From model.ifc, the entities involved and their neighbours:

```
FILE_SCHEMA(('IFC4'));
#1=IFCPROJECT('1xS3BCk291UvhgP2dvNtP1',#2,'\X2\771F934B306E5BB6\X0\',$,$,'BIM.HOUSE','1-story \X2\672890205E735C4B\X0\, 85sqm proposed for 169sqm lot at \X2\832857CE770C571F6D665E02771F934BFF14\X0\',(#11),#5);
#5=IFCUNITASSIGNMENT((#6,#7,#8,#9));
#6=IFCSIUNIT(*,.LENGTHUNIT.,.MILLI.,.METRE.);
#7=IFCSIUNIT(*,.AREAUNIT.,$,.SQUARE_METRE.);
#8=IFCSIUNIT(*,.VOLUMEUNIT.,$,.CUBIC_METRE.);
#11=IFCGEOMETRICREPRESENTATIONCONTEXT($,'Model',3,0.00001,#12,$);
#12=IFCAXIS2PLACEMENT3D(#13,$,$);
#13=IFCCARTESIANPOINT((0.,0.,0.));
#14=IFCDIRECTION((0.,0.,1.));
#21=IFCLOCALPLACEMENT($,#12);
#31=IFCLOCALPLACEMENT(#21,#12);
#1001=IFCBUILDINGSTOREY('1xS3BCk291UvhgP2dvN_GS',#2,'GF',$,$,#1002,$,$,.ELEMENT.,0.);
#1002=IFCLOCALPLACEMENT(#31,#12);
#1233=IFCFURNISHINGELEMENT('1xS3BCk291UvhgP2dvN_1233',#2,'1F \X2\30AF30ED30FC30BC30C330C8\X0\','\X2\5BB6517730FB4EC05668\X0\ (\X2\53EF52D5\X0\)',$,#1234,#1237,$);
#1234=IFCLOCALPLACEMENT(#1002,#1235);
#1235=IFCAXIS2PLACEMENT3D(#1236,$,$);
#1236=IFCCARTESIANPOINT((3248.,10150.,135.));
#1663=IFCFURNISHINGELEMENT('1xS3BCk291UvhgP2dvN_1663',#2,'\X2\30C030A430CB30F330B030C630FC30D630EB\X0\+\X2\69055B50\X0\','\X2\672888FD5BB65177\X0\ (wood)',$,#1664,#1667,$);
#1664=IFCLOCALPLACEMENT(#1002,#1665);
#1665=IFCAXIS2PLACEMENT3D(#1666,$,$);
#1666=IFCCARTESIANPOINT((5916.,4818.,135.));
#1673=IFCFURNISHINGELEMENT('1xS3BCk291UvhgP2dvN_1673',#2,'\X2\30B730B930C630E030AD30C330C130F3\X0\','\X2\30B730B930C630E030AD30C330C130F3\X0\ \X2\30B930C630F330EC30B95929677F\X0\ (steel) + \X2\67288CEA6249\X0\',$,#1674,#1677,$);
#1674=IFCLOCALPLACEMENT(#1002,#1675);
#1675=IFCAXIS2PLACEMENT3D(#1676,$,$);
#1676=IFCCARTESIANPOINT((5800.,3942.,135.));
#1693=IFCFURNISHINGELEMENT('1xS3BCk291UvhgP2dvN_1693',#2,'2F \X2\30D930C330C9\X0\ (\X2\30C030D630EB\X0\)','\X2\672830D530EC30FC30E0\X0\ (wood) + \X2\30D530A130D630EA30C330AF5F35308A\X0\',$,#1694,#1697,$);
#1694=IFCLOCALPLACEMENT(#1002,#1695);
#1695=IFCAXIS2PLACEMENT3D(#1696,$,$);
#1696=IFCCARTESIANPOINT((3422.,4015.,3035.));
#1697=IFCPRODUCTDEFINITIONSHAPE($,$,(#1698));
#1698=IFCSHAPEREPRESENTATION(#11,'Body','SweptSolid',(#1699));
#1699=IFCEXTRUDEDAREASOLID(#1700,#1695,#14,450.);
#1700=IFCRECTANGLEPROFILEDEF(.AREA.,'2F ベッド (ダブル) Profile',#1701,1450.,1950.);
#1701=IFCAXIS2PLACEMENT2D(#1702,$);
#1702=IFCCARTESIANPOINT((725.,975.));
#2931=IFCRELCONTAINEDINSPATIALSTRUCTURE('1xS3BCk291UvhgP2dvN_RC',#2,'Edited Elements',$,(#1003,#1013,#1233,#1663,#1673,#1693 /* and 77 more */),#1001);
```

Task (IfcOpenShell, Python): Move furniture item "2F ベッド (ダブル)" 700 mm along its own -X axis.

```python
import ifcopenshell
import ifcopenshell.api.geometry
import ifcopenshell.util.placement

model = ifcopenshell.open("model.ifc")

item = model.by_guid("1xS3BCk291UvhgP2dvN_1693")
matrix = ifcopenshell.util.placement.get_local_placement(item.ObjectPlacement)
matrix[:3, 3] -= matrix[:3, 0] * 700.0
ifcopenshell.api.geometry.edit_object_placement(model, product=item, matrix=matrix, is_si=False)

print(ifcopenshell.util.placement.get_local_placement(item.ObjectPlacement).round(3) + 0.0)

model.write("model_rev.ifc")
```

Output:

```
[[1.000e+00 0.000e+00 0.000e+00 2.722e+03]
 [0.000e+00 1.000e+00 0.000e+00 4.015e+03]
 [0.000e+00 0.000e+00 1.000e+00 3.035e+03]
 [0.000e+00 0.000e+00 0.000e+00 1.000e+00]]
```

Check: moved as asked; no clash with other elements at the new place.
